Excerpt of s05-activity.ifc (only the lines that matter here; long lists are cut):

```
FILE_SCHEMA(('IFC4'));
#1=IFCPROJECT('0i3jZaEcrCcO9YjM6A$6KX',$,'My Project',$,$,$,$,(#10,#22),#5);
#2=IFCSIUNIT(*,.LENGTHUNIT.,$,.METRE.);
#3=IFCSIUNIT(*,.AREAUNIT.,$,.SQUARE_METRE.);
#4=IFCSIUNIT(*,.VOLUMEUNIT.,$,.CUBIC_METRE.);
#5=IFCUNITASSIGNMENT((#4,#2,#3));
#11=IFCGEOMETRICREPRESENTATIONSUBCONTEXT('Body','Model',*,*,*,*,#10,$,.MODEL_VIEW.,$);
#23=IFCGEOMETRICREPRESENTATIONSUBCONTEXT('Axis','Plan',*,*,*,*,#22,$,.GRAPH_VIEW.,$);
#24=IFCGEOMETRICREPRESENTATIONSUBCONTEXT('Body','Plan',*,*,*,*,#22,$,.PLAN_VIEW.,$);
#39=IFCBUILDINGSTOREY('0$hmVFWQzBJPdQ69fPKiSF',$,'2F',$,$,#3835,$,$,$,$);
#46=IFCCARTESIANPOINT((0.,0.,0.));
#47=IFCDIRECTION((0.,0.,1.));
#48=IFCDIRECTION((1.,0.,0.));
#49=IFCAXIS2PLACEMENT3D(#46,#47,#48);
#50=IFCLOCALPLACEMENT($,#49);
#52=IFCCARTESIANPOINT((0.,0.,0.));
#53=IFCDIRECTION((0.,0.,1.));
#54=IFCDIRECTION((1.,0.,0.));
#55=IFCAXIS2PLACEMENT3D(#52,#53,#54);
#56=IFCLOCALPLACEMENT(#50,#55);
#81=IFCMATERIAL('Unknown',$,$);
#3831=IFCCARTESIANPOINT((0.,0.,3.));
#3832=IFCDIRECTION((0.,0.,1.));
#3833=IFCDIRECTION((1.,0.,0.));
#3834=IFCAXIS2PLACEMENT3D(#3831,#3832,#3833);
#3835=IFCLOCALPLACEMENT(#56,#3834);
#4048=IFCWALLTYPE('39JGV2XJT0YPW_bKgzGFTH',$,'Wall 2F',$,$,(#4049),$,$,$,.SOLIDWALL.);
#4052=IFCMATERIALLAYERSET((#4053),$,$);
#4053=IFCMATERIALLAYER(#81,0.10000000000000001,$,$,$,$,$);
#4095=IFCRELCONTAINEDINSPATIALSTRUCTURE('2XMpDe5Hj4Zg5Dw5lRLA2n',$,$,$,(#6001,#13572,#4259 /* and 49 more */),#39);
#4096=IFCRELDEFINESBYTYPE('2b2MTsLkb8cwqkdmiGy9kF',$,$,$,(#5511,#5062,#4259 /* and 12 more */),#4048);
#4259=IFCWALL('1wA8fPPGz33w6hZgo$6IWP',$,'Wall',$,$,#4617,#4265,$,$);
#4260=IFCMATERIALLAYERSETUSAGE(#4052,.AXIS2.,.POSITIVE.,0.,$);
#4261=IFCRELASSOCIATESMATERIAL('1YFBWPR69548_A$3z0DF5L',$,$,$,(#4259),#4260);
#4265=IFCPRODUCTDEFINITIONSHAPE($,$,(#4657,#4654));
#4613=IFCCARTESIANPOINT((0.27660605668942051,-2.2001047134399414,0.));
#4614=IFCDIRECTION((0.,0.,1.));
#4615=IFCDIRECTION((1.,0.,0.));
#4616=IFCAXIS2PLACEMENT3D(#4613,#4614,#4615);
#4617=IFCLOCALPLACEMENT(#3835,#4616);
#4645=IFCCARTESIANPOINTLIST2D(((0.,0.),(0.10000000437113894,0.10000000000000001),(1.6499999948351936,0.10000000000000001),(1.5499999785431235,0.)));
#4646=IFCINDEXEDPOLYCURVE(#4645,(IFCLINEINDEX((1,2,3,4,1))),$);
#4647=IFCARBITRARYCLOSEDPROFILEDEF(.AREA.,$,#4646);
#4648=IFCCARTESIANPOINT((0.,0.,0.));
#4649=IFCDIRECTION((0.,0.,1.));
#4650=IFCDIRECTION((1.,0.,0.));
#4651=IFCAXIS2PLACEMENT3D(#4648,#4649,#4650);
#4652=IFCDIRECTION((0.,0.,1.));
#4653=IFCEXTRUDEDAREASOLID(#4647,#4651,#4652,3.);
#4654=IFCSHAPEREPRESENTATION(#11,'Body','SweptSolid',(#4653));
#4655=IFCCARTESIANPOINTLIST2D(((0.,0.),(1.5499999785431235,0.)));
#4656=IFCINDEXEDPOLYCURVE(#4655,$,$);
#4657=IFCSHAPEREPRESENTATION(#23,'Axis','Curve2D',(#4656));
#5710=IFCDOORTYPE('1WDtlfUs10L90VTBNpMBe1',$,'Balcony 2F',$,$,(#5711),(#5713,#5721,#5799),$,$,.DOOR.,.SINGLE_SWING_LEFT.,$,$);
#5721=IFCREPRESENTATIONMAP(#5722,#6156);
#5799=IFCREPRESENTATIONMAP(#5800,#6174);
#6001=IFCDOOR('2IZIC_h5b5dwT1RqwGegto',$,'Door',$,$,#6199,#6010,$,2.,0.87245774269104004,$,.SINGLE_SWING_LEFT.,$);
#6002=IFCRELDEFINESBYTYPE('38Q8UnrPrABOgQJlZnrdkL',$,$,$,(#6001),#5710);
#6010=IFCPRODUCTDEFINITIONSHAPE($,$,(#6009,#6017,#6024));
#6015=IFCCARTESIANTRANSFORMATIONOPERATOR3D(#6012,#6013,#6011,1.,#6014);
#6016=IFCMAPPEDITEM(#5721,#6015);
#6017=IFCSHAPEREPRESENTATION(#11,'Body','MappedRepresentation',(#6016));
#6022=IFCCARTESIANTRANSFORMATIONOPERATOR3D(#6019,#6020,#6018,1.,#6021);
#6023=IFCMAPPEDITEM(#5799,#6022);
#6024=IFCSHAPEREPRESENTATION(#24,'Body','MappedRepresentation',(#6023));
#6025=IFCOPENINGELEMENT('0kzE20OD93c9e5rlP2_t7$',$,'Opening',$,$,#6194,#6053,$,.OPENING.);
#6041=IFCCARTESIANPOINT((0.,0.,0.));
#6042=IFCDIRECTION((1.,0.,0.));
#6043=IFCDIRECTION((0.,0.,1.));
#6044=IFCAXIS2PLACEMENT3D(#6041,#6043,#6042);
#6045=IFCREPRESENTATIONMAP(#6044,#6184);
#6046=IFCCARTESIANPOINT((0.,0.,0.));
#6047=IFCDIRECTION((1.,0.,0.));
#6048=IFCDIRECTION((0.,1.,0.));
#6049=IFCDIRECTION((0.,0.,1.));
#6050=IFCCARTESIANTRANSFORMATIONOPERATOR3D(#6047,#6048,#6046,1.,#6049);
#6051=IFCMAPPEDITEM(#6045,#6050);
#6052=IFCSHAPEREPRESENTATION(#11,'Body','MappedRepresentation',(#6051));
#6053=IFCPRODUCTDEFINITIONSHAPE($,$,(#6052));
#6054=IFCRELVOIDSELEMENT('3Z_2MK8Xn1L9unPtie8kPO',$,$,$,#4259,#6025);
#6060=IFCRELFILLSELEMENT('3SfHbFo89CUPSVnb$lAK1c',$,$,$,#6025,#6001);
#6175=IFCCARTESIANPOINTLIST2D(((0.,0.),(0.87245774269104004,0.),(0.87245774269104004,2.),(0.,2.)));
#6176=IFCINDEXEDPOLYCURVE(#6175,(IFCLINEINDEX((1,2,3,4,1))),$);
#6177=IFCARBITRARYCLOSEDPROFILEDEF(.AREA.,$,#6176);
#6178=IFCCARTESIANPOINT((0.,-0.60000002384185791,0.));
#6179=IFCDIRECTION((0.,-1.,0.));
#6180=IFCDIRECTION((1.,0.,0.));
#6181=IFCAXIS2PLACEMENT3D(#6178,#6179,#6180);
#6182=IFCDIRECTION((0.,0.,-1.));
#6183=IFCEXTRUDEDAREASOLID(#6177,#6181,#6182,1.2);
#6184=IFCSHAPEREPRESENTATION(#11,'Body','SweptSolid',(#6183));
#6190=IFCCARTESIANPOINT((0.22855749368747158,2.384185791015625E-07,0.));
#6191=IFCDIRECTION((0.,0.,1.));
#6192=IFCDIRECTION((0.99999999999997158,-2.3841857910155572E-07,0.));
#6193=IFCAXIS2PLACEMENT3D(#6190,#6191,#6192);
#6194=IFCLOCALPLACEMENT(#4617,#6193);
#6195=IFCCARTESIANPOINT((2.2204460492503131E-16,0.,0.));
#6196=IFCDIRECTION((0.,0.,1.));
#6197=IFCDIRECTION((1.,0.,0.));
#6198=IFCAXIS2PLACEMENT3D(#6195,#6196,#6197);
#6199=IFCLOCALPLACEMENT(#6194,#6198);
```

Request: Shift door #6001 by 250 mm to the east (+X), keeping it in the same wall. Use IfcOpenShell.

```python
import ifcopenshell
import ifcopenshell.api.geometry
import ifcopenshell.util.placement
import ifcopenshell.util.unit

model = ifcopenshell.open("s05-activity.ifc")
unit_scale = ifcopenshell.util.unit.calculate_unit_scale(model)

door = model.by_id(6001)
opening = door.FillsVoids[0].RelatingOpeningElement
wall = opening.VoidsElements[0].RelatingBuildingElement

wall_matrix = ifcopenshell.util.placement.get_local_placement(wall.ObjectPlacement)
shift = wall_matrix[:3, 0] * 0.25 / unit_scale
before = ifcopenshell.util.placement.get_local_placement(door.ObjectPlacement)[:3, 3].copy()

# The door is placed relative to its opening, so it follows when the opening moves.
matrix = ifcopenshell.util.placement.get_local_placement(opening.ObjectPlacement)
matrix[:3, 3] += shift
ifcopenshell.api.geometry.edit_object_placement(
    model, product=opening, matrix=matrix, is_si=False, should_transform_children=True
)

after = ifcopenshell.util.placement.get_local_placement(door.ObjectPlacement)[:3, 3]
print("door moved by", (after - before).round(3) + 0.0)

model.write("s05-activity_rev.ifc")
```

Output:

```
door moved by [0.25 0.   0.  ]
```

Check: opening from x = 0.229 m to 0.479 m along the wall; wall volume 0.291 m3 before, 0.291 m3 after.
